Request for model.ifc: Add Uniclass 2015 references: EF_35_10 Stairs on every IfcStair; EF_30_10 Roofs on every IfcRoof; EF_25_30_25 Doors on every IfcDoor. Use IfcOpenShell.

First a look at what the model holds.

```python
import ifcopenshell

model = ifcopenshell.open("model.ifc")
print(model.schema)
print("classifications:", [c.Name for c in model.by_type("IfcClassification")])
for ifc_class in ("IfcDoor", "IfcRoof", "IfcStair", "IfcWall", "IfcWindow"):
    print(ifc_class, len(model.by_type(ifc_class)))
```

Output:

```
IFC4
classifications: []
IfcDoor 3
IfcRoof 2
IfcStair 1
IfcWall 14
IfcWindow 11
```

```python
import ifcopenshell
import ifcopenshell.api.classification

model = ifcopenshell.open("model.ifc")

system = ifcopenshell.api.classification.add_classification(model, classification="Uniclass 2015")

codes = {
    "IfcStair": ("EF_35_10", "Stairs"),
    "IfcRoof": ("EF_30_10", "Roofs"),
    "IfcDoor": ("EF_25_30_25", "Doors"),
}
for ifc_class, (code, name) in codes.items():
    products = model.by_type(ifc_class)
    ifcopenshell.api.classification.add_reference(
        model, products=products, classification=system, identification=code, name=name
    )
    print(code, len(products))

model.write("model_edited.ifc")
```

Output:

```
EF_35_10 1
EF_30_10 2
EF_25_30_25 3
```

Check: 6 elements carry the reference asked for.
